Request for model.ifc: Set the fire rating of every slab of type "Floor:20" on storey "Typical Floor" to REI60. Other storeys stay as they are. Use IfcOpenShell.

First a look at what the model holds.

```python
import ifcopenshell
import ifcopenshell.util.element

model = ifcopenshell.open("model.ifc")
print(model.schema)
storey = next(s for s in model.by_type("IfcBuildingStorey") if s.Name == "Typical Floor")
slabs = [e for e in ifcopenshell.util.element.get_decomposition(storey) if e.is_a("IfcSlab")]
seen = {}
for e in slabs:
    element_type = ifcopenshell.util.element.get_type(e)
    key = (element_type.Name if element_type != e and element_type else None, ifcopenshell.util.element.get_pset(e, "Pset_SlabCommon", "FireRating"))
    seen[key] = seen.get(key, 0) + 1
for (name, value), count in sorted(seen.items(), key=str):
    print(count, "x", name, "|", value)
```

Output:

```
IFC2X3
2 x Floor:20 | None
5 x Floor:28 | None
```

```python
import ifcopenshell
import ifcopenshell.api.pset
import ifcopenshell.util.element

model = ifcopenshell.open("model.ifc")

storey = next(s for s in model.by_type("IfcBuildingStorey") if s.Name == "Typical Floor")
slabs = [e for e in ifcopenshell.util.element.get_decomposition(storey) if e.is_a("IfcSlab")]

count = 0
for e in slabs:
    element_type = ifcopenshell.util.element.get_type(e)
    if element_type in (None, e) or element_type.Name != "Floor:20":
        continue
    # add_pset returns the element's existing set when there is one.
    pset = ifcopenshell.api.pset.add_pset(model, product=e, name="Pset_SlabCommon")
    ifcopenshell.api.pset.edit_pset(model, pset=pset, properties={"FireRating": "REI60"})
    count += 1

print(count, "slabs updated")

model.write("model_v2.ifc")
```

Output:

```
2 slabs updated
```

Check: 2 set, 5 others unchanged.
